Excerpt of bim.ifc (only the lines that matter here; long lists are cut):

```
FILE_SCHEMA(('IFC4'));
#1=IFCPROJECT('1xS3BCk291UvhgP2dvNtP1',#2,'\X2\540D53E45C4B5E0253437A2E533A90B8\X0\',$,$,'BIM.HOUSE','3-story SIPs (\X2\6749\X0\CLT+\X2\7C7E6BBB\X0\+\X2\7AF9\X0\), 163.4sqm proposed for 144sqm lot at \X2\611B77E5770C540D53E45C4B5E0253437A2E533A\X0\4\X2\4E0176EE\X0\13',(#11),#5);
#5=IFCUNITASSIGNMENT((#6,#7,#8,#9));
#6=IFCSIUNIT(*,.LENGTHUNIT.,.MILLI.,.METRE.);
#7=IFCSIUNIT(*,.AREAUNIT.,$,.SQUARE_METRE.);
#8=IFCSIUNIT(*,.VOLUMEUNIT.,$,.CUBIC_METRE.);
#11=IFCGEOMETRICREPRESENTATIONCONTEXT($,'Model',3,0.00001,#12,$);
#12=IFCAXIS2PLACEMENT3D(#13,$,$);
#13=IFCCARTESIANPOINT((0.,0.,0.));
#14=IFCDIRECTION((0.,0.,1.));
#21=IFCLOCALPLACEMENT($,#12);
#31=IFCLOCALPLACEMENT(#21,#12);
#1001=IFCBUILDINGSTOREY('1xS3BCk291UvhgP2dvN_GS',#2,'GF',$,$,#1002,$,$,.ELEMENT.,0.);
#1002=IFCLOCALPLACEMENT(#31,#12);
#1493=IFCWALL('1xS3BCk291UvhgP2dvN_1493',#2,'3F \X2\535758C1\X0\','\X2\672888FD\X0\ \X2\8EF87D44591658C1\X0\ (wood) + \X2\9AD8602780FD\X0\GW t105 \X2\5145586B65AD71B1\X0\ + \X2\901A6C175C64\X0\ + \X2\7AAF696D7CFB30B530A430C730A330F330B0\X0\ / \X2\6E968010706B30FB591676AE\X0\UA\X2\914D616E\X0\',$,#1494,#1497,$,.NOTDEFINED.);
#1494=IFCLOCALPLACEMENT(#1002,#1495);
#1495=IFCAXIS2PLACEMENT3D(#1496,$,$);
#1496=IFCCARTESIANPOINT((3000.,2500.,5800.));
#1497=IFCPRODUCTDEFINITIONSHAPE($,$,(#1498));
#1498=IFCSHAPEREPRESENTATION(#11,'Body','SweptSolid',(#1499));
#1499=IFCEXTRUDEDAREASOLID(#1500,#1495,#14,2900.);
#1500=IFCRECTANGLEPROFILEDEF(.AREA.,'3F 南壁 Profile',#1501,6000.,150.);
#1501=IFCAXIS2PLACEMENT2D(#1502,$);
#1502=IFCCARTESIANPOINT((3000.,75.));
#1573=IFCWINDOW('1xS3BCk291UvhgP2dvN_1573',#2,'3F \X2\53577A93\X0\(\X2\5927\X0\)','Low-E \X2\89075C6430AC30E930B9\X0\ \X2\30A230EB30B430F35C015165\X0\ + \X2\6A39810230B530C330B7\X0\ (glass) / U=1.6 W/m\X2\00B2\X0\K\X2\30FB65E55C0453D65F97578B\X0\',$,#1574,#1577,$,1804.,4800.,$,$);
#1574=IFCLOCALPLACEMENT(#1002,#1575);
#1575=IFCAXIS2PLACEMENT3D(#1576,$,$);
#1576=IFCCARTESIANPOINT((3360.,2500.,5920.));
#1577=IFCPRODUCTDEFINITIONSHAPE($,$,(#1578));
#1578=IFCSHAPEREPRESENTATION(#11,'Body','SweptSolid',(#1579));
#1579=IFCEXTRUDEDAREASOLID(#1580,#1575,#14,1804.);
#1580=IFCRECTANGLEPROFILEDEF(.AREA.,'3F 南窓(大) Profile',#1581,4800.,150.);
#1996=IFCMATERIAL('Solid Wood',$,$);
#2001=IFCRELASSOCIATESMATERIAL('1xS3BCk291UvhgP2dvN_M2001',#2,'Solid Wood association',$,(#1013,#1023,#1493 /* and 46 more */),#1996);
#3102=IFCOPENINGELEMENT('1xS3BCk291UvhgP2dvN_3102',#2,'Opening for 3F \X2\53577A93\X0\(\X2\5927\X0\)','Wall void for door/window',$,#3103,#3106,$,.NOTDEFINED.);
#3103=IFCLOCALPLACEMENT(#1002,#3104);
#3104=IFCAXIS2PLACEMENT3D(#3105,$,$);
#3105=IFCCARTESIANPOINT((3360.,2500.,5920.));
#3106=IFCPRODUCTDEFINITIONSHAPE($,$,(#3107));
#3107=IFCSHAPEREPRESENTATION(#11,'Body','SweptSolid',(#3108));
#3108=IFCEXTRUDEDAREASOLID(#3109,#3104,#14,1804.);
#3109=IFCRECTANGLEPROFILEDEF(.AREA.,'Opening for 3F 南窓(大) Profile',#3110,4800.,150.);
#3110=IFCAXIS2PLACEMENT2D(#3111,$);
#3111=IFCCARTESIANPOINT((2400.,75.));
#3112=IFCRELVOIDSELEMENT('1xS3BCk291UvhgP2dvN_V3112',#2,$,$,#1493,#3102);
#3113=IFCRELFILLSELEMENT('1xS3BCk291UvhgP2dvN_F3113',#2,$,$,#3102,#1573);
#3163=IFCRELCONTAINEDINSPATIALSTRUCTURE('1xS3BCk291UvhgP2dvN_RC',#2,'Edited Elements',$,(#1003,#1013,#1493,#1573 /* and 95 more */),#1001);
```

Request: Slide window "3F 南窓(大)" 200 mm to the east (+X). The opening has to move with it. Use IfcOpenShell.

```python
import ifcopenshell
import ifcopenshell.api.geometry
import ifcopenshell.util.placement
import ifcopenshell.util.unit

model = ifcopenshell.open("bim.ifc")
unit_scale = ifcopenshell.util.unit.calculate_unit_scale(model)

window = model.by_guid("1xS3BCk291UvhgP2dvN_1573")
opening = window.FillsVoids[0].RelatingOpeningElement
wall = opening.VoidsElements[0].RelatingBuildingElement

wall_matrix = ifcopenshell.util.placement.get_local_placement(wall.ObjectPlacement)
shift = wall_matrix[:3, 0] * 0.2 / unit_scale
before = ifcopenshell.util.placement.get_local_placement(window.ObjectPlacement)[:3, 3].copy()

# The window is not placed relative to its opening, so move both.
for product in (opening, window):
    matrix = ifcopenshell.util.placement.get_local_placement(product.ObjectPlacement)
    matrix[:3, 3] += shift
    ifcopenshell.api.geometry.edit_object_placement(model, product=product, matrix=matrix, is_si=False)

after = ifcopenshell.util.placement.get_local_placement(window.ObjectPlacement)[:3, 3]
print("window moved by", (after - before).round(3) + 0.0)

model.write("bim_v2.ifc")
```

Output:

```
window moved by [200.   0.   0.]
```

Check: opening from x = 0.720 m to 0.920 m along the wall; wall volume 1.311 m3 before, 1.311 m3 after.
